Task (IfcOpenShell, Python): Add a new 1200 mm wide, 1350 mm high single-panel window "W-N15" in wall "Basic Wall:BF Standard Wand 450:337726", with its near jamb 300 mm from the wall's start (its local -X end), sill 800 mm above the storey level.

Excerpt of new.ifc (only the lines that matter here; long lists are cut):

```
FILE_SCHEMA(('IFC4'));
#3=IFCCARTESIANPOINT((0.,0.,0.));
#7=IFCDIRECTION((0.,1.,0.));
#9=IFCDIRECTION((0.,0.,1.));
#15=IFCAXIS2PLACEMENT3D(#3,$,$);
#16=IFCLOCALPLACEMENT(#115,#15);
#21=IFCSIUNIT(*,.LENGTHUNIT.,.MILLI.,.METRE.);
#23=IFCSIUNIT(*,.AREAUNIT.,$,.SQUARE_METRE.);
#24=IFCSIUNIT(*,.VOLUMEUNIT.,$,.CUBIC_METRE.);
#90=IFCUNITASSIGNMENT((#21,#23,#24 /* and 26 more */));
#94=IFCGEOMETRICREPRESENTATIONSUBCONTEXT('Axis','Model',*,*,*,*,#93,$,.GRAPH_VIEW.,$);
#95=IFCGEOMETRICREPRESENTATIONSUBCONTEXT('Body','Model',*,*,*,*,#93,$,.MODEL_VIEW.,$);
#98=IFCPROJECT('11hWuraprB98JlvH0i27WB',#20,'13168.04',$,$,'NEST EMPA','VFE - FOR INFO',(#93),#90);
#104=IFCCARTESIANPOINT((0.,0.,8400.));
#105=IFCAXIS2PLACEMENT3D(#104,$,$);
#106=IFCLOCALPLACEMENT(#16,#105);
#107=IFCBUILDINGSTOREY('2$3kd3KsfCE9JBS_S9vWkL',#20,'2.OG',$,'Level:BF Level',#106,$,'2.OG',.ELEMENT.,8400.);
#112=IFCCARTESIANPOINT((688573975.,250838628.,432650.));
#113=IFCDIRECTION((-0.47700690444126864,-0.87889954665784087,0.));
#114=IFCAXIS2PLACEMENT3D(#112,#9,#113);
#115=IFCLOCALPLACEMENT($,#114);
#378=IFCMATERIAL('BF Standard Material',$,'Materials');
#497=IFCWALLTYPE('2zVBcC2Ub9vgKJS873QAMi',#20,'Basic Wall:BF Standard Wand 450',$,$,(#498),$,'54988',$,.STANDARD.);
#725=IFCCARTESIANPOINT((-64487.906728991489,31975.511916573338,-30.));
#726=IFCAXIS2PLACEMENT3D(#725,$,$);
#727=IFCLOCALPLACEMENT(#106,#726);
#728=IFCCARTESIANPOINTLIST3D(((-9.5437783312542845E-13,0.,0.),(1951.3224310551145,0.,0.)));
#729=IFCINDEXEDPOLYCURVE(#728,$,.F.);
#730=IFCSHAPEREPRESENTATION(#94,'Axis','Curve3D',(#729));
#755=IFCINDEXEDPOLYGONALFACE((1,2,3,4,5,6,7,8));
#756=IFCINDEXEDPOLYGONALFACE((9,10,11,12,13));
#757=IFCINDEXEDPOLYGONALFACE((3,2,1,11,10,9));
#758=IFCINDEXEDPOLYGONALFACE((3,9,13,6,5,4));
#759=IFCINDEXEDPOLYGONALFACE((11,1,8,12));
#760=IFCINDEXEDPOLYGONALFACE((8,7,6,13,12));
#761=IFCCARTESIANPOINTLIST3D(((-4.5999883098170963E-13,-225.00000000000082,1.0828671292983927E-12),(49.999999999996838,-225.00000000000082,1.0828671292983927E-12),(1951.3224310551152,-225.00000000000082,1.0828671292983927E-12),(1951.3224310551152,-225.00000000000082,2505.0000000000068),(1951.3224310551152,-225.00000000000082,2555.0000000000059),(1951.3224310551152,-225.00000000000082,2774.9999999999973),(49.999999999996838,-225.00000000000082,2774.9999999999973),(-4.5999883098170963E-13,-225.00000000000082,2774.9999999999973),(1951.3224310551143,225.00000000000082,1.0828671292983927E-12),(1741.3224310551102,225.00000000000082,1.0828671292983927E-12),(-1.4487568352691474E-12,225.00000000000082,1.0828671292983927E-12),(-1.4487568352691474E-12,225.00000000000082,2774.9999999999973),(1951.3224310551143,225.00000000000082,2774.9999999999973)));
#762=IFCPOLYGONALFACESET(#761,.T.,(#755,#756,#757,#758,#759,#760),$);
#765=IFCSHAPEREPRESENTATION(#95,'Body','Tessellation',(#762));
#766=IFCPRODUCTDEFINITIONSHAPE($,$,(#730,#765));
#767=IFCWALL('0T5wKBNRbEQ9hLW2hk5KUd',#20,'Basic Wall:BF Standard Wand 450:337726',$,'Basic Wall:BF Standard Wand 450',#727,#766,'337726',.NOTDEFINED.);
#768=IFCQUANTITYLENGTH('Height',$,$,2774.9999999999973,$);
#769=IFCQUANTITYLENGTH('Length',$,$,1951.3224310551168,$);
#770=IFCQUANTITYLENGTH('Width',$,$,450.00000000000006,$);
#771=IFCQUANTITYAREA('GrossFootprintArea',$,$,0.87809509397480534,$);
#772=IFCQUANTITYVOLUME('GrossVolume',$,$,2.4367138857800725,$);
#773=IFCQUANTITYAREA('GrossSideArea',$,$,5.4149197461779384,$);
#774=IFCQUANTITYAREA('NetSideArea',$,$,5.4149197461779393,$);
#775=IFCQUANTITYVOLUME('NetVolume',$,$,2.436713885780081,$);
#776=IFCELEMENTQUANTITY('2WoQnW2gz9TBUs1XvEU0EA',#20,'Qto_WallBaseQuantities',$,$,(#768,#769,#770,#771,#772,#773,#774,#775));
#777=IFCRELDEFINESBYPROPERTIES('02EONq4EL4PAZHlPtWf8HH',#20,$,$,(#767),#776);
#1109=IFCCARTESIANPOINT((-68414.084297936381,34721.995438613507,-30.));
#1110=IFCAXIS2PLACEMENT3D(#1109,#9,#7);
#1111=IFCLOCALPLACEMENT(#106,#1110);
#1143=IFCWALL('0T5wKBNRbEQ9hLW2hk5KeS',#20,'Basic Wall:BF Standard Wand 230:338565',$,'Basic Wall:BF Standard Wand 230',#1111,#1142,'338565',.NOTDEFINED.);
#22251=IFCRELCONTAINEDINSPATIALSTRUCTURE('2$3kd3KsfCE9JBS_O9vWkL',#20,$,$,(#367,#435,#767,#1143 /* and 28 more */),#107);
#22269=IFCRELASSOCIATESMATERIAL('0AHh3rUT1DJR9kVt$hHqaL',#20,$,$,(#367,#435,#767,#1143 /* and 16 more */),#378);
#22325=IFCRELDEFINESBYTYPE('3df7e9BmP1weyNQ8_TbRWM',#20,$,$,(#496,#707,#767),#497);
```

```python
import numpy as np
import ifcopenshell
import ifcopenshell.api.feature
import ifcopenshell.api.geometry
import ifcopenshell.api.pset
import ifcopenshell.api.root
import ifcopenshell.api.spatial
import ifcopenshell.geom
import ifcopenshell.util.element
import ifcopenshell.util.placement
import ifcopenshell.util.representation
import ifcopenshell.util.shape
import ifcopenshell.util.unit

model = ifcopenshell.open("new.ifc")
unit_scale = ifcopenshell.util.unit.calculate_unit_scale(model)
area_scale = ifcopenshell.util.unit.calculate_unit_scale(model, "AREAUNIT")
volume_scale = ifcopenshell.util.unit.calculate_unit_scale(model, "VOLUMEUNIT")
settings = ifcopenshell.geom.settings()


def volume(element):
    """Net volume in cubic metres, openings subtracted."""
    shape = ifcopenshell.geom.create_shape(settings, element)
    return ifcopenshell.util.shape.get_volume(shape.geometry)


wall = model.by_id(767)
storey = ifcopenshell.util.element.get_container(wall, ifc_class="IfcBuildingStorey")
context = ifcopenshell.util.representation.get_context(model, "Model", "Body", "MODEL_VIEW")
before = volume(wall)

width, height, from_end, sill = 1.2, 1.35, 0.3, 0.8  # metres

# The wall runs along its own X axis, and the end named is its -X end.
wall_shape = ifcopenshell.geom.create_shape(settings, wall)
x, y, z = ifcopenshell.util.shape.get_vertices(wall_shape.geometry).T
start = x.min() + from_end
face, thickness = float(y.min()), float(y.max() - y.min())
wall_matrix = ifcopenshell.util.placement.get_local_placement(wall.ObjectPlacement)
level = ifcopenshell.util.placement.get_local_placement(storey.ObjectPlacement)[2, 3]


def in_wall(x, y):
    """Placement at x, y metres in the wall's axes, at sill height."""
    matrix = wall_matrix.copy()
    matrix[:, 3] = wall_matrix @ np.array([x / unit_scale, y / unit_scale, 0.0, 1.0])
    matrix[2, 3] = level + sill / unit_scale
    return matrix


# Opening: a box that overshoots both wall faces by 50 mm.
opening = ifcopenshell.api.root.create_entity(model, ifc_class="IfcOpeningElement", predefined_type="OPENING")
box = ifcopenshell.api.geometry.add_wall_representation(
    model, context=context, length=width, height=height, thickness=thickness + 0.1
)
ifcopenshell.api.geometry.assign_representation(model, product=opening, representation=box)
ifcopenshell.api.geometry.edit_object_placement(model, product=opening, matrix=in_wall(start, face - 0.05), is_si=False)
ifcopenshell.api.feature.add_feature(model, feature=opening, element=wall)

window = ifcopenshell.api.root.create_entity(model, ifc_class="IfcWindow", name="W-N15", predefined_type="WINDOW")
window.OverallWidth, window.OverallHeight = width / unit_scale, height / unit_scale
window.PartitioningType = "SINGLE_PANEL"
body = ifcopenshell.api.geometry.add_window_representation(
    model,
    context=context,
    overall_width=window.OverallWidth,
    overall_height=window.OverallHeight,
    partition_type="SINGLE_PANEL",
)
ifcopenshell.api.geometry.assign_representation(model, product=window, representation=body)
ifcopenshell.api.spatial.assign_container(model, products=[window], relating_structure=storey)
ifcopenshell.api.feature.add_filling(model, opening=opening, element=window)

# Centre the window in the wall's thickness.
ifcopenshell.api.geometry.edit_object_placement(model, product=window, matrix=in_wall(start, face), is_si=False)
window_shape = ifcopenshell.geom.create_shape(settings, window)
depth = ifcopenshell.util.shape.get_vertices(window_shape.geometry)[:, 1]
offset = face + thickness / 2 - (depth.min() + depth.max()) / 2
ifcopenshell.api.geometry.edit_object_placement(model, product=window, matrix=in_wall(start, offset), is_si=False)

after = volume(wall)

# Update the wall's stored quantities.
qto = model.by_id(ifcopenshell.util.element.get_pset(wall, "Qto_WallBaseQuantities", should_inherit=False)["id"])
ifcopenshell.api.pset.edit_qto(model, qto=qto, properties={
    "NetSideArea": after / thickness / area_scale,
    "NetVolume": after / volume_scale,
})

print(f"wall volume {before:.3f} -> {after:.3f} m3")

model.write("new_updated.ifc")
```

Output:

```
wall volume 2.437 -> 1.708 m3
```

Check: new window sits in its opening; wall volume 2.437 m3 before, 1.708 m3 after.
